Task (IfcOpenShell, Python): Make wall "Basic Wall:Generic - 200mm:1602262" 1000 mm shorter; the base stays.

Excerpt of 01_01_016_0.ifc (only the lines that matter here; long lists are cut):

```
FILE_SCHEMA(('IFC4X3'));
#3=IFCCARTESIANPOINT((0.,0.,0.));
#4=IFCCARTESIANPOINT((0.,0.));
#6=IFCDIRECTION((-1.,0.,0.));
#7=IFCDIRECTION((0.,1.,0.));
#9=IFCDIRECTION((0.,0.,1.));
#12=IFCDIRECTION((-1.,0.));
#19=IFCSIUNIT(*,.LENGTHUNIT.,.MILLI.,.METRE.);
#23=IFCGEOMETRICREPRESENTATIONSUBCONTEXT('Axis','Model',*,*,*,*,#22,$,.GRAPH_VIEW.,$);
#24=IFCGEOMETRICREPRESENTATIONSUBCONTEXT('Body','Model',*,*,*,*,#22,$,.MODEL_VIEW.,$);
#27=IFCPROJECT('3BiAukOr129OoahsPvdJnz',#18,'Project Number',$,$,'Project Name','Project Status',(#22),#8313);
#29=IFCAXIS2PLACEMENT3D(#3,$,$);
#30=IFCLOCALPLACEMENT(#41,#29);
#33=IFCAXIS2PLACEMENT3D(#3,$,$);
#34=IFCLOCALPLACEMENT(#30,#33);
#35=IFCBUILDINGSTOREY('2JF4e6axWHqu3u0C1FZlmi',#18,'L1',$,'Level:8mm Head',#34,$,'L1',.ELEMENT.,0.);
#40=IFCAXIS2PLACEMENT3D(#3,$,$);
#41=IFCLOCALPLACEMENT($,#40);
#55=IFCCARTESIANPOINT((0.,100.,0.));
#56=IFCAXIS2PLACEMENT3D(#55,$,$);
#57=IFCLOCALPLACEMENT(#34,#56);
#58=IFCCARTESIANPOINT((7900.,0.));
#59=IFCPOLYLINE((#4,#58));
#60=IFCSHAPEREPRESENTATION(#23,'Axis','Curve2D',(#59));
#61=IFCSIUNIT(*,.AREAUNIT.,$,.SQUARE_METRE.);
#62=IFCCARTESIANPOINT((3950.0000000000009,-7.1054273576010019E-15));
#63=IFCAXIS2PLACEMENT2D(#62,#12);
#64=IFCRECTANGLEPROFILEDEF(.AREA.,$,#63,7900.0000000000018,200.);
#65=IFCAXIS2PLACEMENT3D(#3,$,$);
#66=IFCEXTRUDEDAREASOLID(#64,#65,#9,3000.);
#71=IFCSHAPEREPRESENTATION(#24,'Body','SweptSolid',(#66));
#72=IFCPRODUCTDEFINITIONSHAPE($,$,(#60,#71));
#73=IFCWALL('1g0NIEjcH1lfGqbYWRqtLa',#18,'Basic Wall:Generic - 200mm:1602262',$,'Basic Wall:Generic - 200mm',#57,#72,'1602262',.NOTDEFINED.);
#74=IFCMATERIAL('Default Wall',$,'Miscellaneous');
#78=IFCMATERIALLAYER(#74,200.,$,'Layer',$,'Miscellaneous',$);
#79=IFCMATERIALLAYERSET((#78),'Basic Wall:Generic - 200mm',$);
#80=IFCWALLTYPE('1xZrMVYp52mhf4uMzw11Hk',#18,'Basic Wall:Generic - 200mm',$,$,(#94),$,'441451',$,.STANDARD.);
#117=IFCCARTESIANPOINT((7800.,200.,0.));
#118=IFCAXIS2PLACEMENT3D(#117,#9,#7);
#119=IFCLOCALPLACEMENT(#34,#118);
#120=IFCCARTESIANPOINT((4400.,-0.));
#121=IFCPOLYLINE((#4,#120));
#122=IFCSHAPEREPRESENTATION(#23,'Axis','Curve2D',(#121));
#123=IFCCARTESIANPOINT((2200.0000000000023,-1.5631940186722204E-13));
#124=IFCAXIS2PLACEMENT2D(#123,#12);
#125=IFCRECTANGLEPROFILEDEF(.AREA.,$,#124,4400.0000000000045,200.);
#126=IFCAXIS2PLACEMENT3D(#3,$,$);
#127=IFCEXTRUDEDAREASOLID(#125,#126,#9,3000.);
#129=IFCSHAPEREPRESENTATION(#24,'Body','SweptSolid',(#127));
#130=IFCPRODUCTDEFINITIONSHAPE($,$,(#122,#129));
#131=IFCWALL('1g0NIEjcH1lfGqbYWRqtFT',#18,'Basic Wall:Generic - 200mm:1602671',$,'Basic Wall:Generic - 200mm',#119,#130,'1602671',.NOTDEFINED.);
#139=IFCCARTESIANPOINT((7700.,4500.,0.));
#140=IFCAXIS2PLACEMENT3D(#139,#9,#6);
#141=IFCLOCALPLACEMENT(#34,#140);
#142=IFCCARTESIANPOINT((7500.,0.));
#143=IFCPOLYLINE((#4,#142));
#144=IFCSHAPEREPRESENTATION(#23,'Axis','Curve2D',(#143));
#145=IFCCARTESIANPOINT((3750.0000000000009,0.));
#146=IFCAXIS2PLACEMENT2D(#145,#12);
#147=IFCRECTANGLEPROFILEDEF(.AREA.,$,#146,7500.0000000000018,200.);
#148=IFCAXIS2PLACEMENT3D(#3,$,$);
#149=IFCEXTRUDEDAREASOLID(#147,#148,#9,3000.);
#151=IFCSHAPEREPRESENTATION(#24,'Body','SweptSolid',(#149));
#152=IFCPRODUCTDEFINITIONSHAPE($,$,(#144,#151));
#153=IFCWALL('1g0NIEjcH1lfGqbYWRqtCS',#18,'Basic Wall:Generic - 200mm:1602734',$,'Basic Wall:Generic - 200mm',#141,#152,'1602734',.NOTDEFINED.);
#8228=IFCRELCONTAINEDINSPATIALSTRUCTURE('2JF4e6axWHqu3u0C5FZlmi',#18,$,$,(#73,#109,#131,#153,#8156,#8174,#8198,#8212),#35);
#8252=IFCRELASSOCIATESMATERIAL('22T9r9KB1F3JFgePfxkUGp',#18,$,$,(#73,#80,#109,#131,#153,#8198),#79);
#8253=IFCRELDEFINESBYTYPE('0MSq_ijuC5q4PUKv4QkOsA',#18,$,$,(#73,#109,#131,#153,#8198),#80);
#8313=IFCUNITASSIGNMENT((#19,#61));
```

```python
import ifcopenshell
import ifcopenshell.geom
import ifcopenshell.util.representation
import ifcopenshell.util.shape

model = ifcopenshell.open("01_01_016_0.ifc")
settings = ifcopenshell.geom.settings()


def volume(element):
    """Net volume in cubic metres, openings subtracted."""
    shape = ifcopenshell.geom.create_shape(settings, element)
    return ifcopenshell.util.shape.get_volume(shape.geometry)


wall = model.by_id(73)
before = volume(wall)

body = ifcopenshell.util.representation.get_representation(wall, "Model", "Body")
solid = body.Items[0]
old_height = solid.Depth
solid.Depth -= 1000.0
after = volume(wall)

print(f"height {old_height:g} -> {solid.Depth:g}, volume {before:.3f} -> {after:.3f} m3")

model.write("01_01_016_0_updated.ifc")
```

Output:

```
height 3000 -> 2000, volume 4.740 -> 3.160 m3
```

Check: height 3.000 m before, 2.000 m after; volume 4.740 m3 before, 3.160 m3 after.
